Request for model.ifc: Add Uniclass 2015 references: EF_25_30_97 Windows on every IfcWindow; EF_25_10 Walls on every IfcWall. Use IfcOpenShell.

First a look at what the model holds.

```python
import ifcopenshell

model = ifcopenshell.open("model.ifc")
print(model.schema)
print("classifications:", [c.Name for c in model.by_type("IfcClassification")])
for ifc_class in ("IfcDoor", "IfcRoof", "IfcStair", "IfcWall", "IfcWindow"):
    print(ifc_class, len(model.by_type(ifc_class)))
```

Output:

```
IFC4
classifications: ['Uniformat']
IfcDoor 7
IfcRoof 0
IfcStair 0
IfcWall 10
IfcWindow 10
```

```python
import ifcopenshell
import ifcopenshell.api.classification

model = ifcopenshell.open("model.ifc")

system = ifcopenshell.api.classification.add_classification(model, classification="Uniclass 2015")

codes = {
    "IfcWindow": ("EF_25_30_97", "Windows"),
    "IfcWall": ("EF_25_10", "Walls"),
}
for ifc_class, (code, name) in codes.items():
    products = model.by_type(ifc_class)
    ifcopenshell.api.classification.add_reference(
        model, products=products, classification=system, identification=code, name=name
    )
    print(code, len(products))

model.write("model_rev.ifc")
```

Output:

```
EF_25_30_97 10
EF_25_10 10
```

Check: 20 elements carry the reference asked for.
